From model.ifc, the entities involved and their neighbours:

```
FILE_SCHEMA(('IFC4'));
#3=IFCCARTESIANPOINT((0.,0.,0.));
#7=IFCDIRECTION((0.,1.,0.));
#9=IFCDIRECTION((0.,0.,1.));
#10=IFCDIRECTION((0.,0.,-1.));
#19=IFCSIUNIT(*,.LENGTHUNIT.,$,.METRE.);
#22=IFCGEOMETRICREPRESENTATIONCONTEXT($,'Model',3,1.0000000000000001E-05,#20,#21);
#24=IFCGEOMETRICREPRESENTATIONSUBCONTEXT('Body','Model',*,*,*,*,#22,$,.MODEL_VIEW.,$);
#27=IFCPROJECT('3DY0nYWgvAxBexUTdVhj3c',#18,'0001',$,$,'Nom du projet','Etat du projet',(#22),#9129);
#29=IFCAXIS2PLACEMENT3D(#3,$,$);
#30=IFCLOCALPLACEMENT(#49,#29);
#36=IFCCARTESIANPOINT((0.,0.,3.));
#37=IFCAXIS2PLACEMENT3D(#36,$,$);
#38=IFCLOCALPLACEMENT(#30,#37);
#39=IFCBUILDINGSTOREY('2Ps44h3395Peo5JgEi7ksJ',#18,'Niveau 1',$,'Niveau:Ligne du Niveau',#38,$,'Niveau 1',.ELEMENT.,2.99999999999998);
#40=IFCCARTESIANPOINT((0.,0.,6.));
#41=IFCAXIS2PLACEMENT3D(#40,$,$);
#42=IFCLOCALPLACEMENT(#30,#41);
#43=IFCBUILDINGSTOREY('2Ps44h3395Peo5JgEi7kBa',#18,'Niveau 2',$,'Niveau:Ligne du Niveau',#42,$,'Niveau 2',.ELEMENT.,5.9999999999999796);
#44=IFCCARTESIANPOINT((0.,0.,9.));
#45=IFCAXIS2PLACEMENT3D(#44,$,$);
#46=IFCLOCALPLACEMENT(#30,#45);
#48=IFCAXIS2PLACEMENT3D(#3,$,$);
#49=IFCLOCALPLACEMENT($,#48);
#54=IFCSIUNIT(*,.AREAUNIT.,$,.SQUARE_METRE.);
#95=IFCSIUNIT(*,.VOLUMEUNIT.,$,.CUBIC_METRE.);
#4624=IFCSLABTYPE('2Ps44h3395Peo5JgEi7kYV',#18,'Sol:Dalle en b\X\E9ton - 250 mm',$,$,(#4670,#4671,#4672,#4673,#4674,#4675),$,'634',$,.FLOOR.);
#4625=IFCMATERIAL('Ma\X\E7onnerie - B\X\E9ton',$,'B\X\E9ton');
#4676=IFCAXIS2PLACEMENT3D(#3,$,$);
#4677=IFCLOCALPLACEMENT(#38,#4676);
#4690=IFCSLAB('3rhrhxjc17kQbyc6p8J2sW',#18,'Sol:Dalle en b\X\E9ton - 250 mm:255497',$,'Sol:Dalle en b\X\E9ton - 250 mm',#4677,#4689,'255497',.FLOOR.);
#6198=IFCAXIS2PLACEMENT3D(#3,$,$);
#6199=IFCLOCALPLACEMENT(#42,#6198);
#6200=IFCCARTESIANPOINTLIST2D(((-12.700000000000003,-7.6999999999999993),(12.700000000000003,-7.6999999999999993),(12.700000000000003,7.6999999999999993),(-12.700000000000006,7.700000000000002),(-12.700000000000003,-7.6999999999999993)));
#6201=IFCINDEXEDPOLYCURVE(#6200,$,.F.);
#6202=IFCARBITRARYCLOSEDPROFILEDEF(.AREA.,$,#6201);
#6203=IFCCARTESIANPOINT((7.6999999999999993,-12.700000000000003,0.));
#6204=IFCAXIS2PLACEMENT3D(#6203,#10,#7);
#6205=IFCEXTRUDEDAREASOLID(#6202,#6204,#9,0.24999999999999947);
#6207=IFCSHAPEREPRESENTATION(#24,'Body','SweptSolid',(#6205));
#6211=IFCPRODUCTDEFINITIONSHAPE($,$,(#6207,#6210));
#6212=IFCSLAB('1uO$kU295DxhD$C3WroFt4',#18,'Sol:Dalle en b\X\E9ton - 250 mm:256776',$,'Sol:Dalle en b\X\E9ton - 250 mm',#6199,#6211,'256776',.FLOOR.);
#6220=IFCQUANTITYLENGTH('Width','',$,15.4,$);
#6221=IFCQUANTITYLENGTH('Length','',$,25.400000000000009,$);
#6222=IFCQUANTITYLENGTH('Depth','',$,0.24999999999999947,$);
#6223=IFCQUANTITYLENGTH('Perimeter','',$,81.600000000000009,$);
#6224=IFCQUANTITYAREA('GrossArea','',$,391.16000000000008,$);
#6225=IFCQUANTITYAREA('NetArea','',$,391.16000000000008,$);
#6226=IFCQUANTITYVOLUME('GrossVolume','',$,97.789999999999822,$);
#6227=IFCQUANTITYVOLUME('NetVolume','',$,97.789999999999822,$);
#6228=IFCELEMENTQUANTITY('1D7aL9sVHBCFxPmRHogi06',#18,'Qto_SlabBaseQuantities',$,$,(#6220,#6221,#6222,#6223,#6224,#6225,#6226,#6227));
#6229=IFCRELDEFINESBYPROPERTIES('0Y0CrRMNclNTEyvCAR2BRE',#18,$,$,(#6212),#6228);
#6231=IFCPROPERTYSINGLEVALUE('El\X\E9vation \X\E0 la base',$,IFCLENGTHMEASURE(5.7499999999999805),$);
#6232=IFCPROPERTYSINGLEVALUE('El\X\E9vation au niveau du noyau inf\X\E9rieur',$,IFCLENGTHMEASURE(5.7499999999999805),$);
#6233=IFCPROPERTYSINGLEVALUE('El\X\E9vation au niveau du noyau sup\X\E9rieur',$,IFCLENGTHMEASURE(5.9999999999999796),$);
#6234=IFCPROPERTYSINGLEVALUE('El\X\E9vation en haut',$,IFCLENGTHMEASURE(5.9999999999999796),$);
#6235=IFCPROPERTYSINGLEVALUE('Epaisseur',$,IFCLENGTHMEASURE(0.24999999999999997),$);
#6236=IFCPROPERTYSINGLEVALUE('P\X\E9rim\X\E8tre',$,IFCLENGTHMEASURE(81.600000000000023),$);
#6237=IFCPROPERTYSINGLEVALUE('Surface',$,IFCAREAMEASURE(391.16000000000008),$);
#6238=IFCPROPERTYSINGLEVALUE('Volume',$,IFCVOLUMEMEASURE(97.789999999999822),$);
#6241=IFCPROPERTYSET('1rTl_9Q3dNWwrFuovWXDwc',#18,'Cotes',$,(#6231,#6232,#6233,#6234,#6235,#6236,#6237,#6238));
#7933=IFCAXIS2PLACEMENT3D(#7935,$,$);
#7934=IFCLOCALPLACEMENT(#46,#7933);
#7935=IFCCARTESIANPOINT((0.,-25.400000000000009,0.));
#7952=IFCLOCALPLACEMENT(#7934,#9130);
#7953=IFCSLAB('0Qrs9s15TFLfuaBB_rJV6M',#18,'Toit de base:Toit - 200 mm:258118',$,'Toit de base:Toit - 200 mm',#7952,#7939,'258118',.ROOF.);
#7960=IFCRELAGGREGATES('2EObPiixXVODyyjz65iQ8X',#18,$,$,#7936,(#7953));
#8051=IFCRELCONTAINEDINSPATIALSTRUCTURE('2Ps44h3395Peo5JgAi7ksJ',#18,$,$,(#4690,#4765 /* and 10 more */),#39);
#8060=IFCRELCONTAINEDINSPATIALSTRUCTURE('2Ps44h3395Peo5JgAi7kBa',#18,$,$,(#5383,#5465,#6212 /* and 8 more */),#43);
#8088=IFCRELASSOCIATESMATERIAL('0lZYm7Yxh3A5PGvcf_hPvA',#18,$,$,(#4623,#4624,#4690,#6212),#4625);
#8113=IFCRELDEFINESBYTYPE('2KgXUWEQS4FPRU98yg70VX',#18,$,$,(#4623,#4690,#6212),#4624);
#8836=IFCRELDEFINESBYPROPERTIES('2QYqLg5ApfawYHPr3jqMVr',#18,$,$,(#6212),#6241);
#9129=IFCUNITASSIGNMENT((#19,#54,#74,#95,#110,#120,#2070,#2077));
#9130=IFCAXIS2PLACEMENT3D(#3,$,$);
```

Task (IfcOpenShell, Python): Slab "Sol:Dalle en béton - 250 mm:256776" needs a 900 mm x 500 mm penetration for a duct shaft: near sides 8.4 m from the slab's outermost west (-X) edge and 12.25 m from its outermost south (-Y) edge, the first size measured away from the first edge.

```python
import numpy as np
import ifcopenshell
import ifcopenshell.api.feature
import ifcopenshell.api.geometry
import ifcopenshell.api.pset
import ifcopenshell.api.root
import ifcopenshell.geom
import ifcopenshell.util.element
import ifcopenshell.util.placement
import ifcopenshell.util.representation
import ifcopenshell.util.shape
import ifcopenshell.util.unit

model = ifcopenshell.open("model.ifc")
unit_scale = ifcopenshell.util.unit.calculate_unit_scale(model)
area_scale = ifcopenshell.util.unit.calculate_unit_scale(model, "AREAUNIT")
volume_scale = ifcopenshell.util.unit.calculate_unit_scale(model, "VOLUMEUNIT")
settings = ifcopenshell.geom.settings()


def volume(element):
    """Net volume in cubic metres, openings subtracted."""
    shape = ifcopenshell.geom.create_shape(settings, element)
    return ifcopenshell.util.shape.get_volume(shape.geometry)


slab = model.by_id(6212)
before = volume(slab)

# Extent in the slab's own axes, in metres. The edges named are its -X and -Y sides.
slab_shape = ifcopenshell.geom.create_shape(settings, slab)
vertices = ifcopenshell.util.shape.get_vertices(slab_shape.geometry)
x_min, y_min, bottom = vertices.min(axis=0)
top = vertices[:, 2].max()

opening = ifcopenshell.api.root.create_entity(model, ifc_class="IfcOpeningElement", name="Duct shaft opening", predefined_type="OPENING")
context = ifcopenshell.util.representation.get_context(model, "Model", "Body", "MODEL_VIEW")
width, depth = 0.9, 0.5
outline = [(0.0, 0.0), (width, 0.0), (width, depth), (0.0, depth), (0.0, 0.0)]
# Overshoot both faces by 50 mm so the cut is clean.
shape = ifcopenshell.api.geometry.add_slab_representation(
    model, context=context, depth=top - bottom + 0.1, polyline=outline
)
ifcopenshell.api.geometry.assign_representation(model, product=opening, representation=shape)

matrix = ifcopenshell.util.placement.get_local_placement(slab.ObjectPlacement)
matrix[:, 3] = matrix @ np.append(np.array([x_min + 8.4, y_min + 12.25, bottom - 0.05]) / unit_scale, 1.0)
ifcopenshell.api.geometry.edit_object_placement(model, product=opening, matrix=matrix, is_si=False)
ifcopenshell.api.feature.add_feature(model, feature=opening, element=slab)

after = volume(slab)

# Update the slab's stored quantities.
qto = model.by_id(ifcopenshell.util.element.get_pset(slab, "Qto_SlabBaseQuantities", should_inherit=False)["id"])
ifcopenshell.api.pset.edit_qto(model, qto=qto, properties={
    "NetArea": after / (top - bottom) / area_scale,
    "NetVolume": after / volume_scale,
})
pset = model.by_id(ifcopenshell.util.element.get_pset(slab, "Cotes", should_inherit=False)["id"])
ifcopenshell.api.pset.edit_pset(model, pset=pset, properties={
    "Surface": model.create_entity("IfcAreaMeasure", after / (top - bottom) / area_scale),
    "Volume": model.create_entity("IfcVolumeMeasure", after / volume_scale),
})

print(f"slab volume {before:.3f} -> {after:.3f} m3")

model.write("model_rev.ifc")
```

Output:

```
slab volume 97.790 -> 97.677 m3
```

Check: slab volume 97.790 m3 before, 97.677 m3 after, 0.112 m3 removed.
